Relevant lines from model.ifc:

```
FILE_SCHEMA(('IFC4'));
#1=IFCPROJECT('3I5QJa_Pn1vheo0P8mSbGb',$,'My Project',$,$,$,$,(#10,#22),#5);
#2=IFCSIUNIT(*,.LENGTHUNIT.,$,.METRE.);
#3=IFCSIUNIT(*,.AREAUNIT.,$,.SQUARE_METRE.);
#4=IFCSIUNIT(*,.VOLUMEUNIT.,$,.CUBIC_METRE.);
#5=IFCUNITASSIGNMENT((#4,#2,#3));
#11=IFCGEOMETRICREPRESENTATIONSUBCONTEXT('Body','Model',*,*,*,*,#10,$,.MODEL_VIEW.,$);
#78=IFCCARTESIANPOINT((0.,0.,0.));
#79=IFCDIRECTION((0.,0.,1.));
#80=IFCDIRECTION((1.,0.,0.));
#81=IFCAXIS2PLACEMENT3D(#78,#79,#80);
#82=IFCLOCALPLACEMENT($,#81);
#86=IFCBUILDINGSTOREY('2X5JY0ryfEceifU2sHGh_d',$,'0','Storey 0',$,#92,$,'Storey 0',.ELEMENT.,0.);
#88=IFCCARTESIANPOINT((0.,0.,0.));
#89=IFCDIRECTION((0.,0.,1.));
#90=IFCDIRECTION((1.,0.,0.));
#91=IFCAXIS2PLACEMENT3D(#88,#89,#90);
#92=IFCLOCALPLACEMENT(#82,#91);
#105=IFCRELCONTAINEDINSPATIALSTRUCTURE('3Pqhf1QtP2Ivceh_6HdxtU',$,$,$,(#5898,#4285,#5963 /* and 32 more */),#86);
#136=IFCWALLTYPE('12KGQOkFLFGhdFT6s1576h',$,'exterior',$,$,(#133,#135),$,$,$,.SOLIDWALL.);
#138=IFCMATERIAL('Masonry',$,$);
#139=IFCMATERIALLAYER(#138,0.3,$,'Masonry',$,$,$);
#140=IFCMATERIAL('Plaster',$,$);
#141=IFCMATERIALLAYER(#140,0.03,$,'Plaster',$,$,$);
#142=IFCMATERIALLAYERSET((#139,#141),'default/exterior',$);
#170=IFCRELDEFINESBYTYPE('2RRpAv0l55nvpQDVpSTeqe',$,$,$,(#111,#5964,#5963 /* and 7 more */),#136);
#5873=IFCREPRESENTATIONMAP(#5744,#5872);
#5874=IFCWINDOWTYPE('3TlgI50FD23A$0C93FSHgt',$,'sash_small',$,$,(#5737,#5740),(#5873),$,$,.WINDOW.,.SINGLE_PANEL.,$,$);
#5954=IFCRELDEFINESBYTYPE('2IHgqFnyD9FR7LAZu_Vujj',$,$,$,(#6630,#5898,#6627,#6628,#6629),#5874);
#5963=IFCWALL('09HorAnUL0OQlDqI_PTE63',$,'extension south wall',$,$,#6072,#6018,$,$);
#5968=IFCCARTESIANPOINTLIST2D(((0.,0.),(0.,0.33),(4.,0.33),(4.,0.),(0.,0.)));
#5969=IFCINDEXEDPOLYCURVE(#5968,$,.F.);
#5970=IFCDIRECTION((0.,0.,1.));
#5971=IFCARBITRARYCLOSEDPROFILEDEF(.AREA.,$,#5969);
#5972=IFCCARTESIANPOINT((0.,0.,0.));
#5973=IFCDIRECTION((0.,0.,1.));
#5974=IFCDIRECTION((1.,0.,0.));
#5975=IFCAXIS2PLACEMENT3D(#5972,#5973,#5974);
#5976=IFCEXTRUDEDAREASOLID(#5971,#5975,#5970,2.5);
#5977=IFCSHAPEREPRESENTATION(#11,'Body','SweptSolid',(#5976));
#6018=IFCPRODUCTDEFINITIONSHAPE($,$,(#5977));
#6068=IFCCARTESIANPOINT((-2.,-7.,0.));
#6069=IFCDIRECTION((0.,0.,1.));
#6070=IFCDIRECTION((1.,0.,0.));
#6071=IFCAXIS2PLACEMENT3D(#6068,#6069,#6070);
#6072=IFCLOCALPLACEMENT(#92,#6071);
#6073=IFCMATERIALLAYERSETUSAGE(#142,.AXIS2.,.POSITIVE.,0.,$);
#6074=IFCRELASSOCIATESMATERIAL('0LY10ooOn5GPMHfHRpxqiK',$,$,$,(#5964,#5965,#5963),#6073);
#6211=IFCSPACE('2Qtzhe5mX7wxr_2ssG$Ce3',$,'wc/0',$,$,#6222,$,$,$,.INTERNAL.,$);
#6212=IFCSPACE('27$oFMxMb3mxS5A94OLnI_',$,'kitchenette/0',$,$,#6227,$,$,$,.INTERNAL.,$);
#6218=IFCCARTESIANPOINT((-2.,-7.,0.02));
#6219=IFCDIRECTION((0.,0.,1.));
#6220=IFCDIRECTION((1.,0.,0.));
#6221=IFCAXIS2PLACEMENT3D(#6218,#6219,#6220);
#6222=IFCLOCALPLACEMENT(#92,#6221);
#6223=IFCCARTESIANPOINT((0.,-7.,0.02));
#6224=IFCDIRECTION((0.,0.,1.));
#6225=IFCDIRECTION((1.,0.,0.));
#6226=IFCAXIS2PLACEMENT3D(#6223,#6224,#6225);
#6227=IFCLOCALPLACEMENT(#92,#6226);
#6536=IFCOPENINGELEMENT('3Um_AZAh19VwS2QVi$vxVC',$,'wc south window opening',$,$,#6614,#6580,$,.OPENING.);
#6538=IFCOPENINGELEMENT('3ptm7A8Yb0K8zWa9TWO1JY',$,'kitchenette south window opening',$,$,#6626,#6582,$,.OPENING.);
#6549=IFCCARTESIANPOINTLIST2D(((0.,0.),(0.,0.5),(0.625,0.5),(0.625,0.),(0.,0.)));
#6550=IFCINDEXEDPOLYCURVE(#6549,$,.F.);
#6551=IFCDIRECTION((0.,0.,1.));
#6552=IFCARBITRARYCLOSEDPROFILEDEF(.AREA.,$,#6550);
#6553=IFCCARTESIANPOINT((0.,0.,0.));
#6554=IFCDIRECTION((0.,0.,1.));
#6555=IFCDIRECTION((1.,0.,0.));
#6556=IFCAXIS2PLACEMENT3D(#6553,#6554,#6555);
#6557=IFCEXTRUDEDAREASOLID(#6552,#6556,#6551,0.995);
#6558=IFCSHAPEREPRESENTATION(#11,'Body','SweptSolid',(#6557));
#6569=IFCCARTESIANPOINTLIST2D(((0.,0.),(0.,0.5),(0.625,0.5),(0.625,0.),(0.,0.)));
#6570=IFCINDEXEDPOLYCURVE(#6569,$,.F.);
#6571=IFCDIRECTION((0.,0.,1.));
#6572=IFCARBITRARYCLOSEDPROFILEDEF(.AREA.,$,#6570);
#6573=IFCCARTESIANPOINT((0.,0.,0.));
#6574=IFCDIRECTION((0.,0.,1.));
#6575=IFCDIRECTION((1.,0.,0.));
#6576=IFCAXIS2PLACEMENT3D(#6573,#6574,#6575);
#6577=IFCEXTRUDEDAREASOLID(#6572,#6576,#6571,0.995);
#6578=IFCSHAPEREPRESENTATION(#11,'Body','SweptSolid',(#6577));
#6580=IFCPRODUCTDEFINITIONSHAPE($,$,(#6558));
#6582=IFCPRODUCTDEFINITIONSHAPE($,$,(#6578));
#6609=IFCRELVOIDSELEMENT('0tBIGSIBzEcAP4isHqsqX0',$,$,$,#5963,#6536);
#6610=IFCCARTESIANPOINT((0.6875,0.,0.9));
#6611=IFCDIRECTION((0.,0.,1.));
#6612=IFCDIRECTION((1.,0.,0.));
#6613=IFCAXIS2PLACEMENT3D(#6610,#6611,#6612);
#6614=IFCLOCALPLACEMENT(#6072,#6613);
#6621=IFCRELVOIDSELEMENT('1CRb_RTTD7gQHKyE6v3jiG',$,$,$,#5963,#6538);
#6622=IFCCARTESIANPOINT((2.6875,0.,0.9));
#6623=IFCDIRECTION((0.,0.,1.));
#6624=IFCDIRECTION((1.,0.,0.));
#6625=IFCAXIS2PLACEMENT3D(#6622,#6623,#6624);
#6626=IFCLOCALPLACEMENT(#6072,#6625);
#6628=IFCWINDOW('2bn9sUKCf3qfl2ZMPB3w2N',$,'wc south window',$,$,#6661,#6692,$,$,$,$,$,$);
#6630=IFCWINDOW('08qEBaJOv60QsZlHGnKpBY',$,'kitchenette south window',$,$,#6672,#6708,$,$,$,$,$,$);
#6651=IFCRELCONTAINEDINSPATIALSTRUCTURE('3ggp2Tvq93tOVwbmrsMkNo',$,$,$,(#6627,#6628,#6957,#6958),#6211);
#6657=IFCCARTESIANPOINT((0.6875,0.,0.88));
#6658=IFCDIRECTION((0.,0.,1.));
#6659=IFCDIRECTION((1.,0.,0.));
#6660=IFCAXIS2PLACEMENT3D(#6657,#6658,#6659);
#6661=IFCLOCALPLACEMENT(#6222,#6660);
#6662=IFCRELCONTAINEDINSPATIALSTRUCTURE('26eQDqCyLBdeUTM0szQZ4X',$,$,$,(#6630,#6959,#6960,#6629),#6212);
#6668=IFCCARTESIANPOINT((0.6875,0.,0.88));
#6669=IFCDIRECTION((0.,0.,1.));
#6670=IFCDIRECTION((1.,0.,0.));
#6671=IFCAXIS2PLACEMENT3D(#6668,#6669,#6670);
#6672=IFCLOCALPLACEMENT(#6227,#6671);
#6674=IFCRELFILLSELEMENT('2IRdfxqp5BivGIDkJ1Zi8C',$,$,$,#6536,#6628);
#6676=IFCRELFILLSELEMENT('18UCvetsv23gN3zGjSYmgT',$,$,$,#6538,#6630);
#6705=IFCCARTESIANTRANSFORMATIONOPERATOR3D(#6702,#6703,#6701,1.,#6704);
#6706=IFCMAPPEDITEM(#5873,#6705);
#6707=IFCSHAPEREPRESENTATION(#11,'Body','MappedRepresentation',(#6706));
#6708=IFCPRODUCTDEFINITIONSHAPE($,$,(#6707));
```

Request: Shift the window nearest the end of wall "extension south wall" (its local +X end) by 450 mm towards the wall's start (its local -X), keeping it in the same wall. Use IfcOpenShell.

```python
import ifcopenshell
import ifcopenshell.api.geometry
import ifcopenshell.util.placement
import ifcopenshell.util.unit

model = ifcopenshell.open("model.ifc")
unit_scale = ifcopenshell.util.unit.calculate_unit_scale(model)

window = model.by_id(6630)
opening = window.FillsVoids[0].RelatingOpeningElement
wall = opening.VoidsElements[0].RelatingBuildingElement

wall_matrix = ifcopenshell.util.placement.get_local_placement(wall.ObjectPlacement)
shift = wall_matrix[:3, 0] * -0.45 / unit_scale
before = ifcopenshell.util.placement.get_local_placement(window.ObjectPlacement)[:3, 3].copy()

# The window is not placed relative to its opening, so move both.
for product in (opening, window):
    matrix = ifcopenshell.util.placement.get_local_placement(product.ObjectPlacement)
    matrix[:3, 3] += shift
    ifcopenshell.api.geometry.edit_object_placement(model, product=product, matrix=matrix, is_si=False)

after = ifcopenshell.util.placement.get_local_placement(window.ObjectPlacement)[:3, 3]
print("window moved by", (after - before).round(3) + 0.0)

model.write("model_rev.ifc")
```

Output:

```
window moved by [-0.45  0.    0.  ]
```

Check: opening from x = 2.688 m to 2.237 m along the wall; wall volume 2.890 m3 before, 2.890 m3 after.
